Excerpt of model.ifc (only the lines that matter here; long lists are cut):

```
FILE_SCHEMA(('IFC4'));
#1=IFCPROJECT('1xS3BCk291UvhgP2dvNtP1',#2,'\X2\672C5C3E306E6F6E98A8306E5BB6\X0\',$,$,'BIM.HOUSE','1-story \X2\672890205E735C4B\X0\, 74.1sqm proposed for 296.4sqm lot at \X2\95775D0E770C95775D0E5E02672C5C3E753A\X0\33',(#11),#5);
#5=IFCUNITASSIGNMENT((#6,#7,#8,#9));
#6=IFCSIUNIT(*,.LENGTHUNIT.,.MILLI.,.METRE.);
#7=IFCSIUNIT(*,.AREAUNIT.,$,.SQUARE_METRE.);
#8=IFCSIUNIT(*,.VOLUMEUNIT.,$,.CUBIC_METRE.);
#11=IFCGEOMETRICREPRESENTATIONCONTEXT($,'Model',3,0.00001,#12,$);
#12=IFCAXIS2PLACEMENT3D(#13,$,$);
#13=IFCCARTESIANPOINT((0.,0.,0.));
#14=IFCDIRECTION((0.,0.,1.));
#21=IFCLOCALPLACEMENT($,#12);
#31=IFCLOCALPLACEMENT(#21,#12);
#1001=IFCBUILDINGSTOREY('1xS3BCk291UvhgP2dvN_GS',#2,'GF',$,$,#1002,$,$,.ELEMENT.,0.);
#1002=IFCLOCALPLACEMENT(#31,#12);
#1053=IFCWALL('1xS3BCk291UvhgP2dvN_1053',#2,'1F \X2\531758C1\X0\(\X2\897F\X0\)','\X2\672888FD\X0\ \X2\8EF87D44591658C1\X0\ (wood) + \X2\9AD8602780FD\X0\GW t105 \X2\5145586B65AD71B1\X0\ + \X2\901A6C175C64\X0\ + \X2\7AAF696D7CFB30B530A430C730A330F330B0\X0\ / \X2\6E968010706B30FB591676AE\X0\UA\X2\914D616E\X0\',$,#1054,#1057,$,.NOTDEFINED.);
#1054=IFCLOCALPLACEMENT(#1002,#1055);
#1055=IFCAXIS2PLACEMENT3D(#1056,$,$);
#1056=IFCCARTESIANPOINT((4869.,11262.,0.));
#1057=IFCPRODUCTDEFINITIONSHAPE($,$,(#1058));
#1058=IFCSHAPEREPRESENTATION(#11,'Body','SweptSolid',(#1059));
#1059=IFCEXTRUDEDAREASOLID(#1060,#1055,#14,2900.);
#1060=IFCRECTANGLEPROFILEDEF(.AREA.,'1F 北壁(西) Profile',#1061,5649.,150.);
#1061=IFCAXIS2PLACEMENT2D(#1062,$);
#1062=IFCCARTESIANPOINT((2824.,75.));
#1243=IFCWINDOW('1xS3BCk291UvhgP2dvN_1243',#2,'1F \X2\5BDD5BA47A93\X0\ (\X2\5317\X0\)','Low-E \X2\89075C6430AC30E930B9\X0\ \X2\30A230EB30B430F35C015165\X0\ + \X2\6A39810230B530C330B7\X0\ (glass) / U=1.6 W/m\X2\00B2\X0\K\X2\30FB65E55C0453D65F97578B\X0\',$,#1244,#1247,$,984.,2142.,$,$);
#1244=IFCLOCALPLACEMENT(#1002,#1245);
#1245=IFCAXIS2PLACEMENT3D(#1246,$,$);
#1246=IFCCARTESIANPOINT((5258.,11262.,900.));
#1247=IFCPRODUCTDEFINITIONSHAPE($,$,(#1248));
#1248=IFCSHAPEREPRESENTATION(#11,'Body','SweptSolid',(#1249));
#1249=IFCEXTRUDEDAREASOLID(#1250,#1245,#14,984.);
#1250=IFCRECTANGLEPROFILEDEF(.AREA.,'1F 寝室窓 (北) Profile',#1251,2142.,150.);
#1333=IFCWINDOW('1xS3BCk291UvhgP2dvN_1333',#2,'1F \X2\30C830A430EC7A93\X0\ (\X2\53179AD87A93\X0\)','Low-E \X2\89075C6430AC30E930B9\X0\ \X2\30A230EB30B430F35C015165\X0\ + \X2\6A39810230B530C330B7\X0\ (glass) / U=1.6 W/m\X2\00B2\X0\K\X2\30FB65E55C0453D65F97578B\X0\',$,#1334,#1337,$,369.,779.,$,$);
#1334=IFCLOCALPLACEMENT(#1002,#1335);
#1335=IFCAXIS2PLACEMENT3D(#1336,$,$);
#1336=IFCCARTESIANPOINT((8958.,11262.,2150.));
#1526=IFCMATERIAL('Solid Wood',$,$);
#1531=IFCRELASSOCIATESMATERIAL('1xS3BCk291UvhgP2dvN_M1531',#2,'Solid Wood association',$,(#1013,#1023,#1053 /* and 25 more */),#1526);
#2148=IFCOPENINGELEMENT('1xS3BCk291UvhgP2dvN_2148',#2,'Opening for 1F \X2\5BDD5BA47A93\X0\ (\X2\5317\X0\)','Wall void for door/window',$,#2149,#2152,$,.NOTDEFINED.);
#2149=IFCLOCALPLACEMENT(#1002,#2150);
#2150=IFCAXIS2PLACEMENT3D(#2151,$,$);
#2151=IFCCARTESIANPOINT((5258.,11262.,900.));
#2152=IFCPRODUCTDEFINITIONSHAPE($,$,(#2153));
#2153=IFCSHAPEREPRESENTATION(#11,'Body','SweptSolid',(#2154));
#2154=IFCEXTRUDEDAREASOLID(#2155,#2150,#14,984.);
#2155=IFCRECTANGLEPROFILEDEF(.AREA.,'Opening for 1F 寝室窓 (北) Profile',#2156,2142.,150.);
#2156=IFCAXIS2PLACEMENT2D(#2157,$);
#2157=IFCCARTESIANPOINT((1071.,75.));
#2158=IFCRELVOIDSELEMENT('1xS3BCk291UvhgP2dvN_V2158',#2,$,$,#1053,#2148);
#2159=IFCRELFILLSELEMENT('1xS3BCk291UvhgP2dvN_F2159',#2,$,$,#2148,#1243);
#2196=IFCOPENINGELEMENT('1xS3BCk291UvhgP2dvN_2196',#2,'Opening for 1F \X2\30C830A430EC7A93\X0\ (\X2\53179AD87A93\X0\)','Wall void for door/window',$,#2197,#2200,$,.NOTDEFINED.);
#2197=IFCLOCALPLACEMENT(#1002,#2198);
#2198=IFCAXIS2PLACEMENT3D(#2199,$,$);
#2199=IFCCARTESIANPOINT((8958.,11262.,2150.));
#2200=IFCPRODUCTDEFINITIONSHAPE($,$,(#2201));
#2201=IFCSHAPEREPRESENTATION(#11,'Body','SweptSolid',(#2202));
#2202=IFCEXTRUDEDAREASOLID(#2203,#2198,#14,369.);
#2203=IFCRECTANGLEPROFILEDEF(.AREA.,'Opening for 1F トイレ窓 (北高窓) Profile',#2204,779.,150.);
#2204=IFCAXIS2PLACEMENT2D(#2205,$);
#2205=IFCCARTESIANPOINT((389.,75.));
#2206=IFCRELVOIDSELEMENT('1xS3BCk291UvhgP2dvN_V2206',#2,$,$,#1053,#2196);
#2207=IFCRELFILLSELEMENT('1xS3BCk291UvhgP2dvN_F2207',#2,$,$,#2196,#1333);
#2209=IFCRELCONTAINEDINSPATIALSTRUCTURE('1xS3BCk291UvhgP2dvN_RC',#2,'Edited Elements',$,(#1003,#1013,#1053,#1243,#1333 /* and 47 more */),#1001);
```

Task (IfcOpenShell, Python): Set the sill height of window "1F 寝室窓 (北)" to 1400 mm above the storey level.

```python
import numpy as np
import ifcopenshell
import ifcopenshell.api.geometry
import ifcopenshell.geom
import ifcopenshell.util.element
import ifcopenshell.util.placement
import ifcopenshell.util.shape
import ifcopenshell.util.unit

model = ifcopenshell.open("model.ifc")
unit_scale = ifcopenshell.util.unit.calculate_unit_scale(model)

window = model.by_guid("1xS3BCk291UvhgP2dvN_1243")
opening = window.FillsVoids[0].RelatingOpeningElement
storey = ifcopenshell.util.element.get_container(window, ifc_class="IfcBuildingStorey")
level = ifcopenshell.util.placement.get_local_placement(storey.ObjectPlacement)[2, 3]

# The opening's origin need not be at the sill, so measure its lowest point.
shape = ifcopenshell.geom.create_shape(ifcopenshell.geom.settings(), opening)
bottom = ifcopenshell.util.shape.get_shape_bottom_elevation(shape, shape.geometry) / unit_scale
dz = level + 1400.0 - bottom

shift = np.array([0.0, 0.0, dz])
# The window is not placed relative to its opening, so move both.
for product in (opening, window):
    matrix = ifcopenshell.util.placement.get_local_placement(product.ObjectPlacement)
    matrix[:3, 3] += shift
    ifcopenshell.api.geometry.edit_object_placement(model, product=product, matrix=matrix, is_si=False)

print(f"moved by {dz * unit_scale:+.3f} m")

model.write("model_v2.ifc")
```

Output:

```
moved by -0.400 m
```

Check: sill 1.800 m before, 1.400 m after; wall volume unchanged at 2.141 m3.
